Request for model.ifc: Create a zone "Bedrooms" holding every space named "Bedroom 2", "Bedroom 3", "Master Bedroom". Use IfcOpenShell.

First a look at what the model holds.

```python
import ifcopenshell

model = ifcopenshell.open("model.ifc")
print(model.schema)
seen = {}
for space in model.by_type("IfcSpace"):
    seen[space.LongName] = seen.get(space.LongName, 0) + 1
for name, count in sorted(seen.items(), key=str):
    print(count, "x", name)
print("zones:", [z.Name for z in model.by_type("IfcZone")][:20])
```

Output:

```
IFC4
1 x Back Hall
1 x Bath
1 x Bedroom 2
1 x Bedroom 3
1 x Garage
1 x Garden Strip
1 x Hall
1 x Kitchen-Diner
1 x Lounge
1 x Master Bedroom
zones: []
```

```python
import ifcopenshell
import ifcopenshell.api.group
import ifcopenshell.api.root

model = ifcopenshell.open("model.ifc")

names = {"Bedroom 2", "Bedroom 3", "Master Bedroom"}
spaces = [s for s in model.by_type("IfcSpace") if s.LongName in names]

zone = ifcopenshell.api.root.create_entity(model, ifc_class="IfcZone", name="Bedrooms")
ifcopenshell.api.group.assign_group(model, products=spaces, group=zone)
print(len(spaces), "spaces in", zone.Name)

model.write("model_edited.ifc")
```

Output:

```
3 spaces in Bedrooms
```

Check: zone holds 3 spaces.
